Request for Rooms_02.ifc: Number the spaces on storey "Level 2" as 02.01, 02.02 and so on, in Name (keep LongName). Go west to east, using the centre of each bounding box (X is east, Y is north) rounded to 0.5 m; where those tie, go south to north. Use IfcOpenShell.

First a look at what the model holds.

```python
import ifcopenshell
import ifcopenshell.util.element
import ifcopenshell.util.placement

model = ifcopenshell.open("Rooms_02.ifc")
print(model.schema)
storey = next(s for s in model.by_type("IfcBuildingStorey") if s.Name == "Level 2")
spaces = [e for e in ifcopenshell.util.element.get_decomposition(storey) if e.is_a("IfcSpace")]
for e in sorted(spaces, key=lambda e: e.id()):
    origin = ifcopenshell.util.placement.get_local_placement(e.ObjectPlacement)[:3, 3]
    print(e.id(), e.Name, e.LongName, origin.round(2) + 0.0, sep=" | ")
```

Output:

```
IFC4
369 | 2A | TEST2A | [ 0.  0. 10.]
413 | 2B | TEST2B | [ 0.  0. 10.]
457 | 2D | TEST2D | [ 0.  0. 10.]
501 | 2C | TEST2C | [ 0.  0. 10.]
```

```python
import ifcopenshell
import ifcopenshell.geom
import ifcopenshell.util.element
import ifcopenshell.util.shape

model = ifcopenshell.open("Rooms_02.ifc")
settings = ifcopenshell.geom.settings()
settings.set("use-world-coords", True)


def centre(element):
    shape = ifcopenshell.geom.create_shape(settings, element)
    return ifcopenshell.util.shape.get_bbox_centroid(shape.geometry)


storey = next(s for s in model.by_type("IfcBuildingStorey") if s.Name == "Level 2")
spaces = [e for e in ifcopenshell.util.element.get_decomposition(storey) if e.is_a("IfcSpace")]

# Insertion points can sit at a corner or the storey origin, so sort by the geometry (in metres).
centres = {e: centre(e) for e in spaces}
spaces.sort(key=lambda e: (round(centres[e][0] / 0.5), centres[e][1]))

for i, e in enumerate(spaces, start=1):
    number = f"02.{i:02d}"
    e.Name = number
    print(e.id(), number)

model.write("Rooms_02_rev.ifc")
```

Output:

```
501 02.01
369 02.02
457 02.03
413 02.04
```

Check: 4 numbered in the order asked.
